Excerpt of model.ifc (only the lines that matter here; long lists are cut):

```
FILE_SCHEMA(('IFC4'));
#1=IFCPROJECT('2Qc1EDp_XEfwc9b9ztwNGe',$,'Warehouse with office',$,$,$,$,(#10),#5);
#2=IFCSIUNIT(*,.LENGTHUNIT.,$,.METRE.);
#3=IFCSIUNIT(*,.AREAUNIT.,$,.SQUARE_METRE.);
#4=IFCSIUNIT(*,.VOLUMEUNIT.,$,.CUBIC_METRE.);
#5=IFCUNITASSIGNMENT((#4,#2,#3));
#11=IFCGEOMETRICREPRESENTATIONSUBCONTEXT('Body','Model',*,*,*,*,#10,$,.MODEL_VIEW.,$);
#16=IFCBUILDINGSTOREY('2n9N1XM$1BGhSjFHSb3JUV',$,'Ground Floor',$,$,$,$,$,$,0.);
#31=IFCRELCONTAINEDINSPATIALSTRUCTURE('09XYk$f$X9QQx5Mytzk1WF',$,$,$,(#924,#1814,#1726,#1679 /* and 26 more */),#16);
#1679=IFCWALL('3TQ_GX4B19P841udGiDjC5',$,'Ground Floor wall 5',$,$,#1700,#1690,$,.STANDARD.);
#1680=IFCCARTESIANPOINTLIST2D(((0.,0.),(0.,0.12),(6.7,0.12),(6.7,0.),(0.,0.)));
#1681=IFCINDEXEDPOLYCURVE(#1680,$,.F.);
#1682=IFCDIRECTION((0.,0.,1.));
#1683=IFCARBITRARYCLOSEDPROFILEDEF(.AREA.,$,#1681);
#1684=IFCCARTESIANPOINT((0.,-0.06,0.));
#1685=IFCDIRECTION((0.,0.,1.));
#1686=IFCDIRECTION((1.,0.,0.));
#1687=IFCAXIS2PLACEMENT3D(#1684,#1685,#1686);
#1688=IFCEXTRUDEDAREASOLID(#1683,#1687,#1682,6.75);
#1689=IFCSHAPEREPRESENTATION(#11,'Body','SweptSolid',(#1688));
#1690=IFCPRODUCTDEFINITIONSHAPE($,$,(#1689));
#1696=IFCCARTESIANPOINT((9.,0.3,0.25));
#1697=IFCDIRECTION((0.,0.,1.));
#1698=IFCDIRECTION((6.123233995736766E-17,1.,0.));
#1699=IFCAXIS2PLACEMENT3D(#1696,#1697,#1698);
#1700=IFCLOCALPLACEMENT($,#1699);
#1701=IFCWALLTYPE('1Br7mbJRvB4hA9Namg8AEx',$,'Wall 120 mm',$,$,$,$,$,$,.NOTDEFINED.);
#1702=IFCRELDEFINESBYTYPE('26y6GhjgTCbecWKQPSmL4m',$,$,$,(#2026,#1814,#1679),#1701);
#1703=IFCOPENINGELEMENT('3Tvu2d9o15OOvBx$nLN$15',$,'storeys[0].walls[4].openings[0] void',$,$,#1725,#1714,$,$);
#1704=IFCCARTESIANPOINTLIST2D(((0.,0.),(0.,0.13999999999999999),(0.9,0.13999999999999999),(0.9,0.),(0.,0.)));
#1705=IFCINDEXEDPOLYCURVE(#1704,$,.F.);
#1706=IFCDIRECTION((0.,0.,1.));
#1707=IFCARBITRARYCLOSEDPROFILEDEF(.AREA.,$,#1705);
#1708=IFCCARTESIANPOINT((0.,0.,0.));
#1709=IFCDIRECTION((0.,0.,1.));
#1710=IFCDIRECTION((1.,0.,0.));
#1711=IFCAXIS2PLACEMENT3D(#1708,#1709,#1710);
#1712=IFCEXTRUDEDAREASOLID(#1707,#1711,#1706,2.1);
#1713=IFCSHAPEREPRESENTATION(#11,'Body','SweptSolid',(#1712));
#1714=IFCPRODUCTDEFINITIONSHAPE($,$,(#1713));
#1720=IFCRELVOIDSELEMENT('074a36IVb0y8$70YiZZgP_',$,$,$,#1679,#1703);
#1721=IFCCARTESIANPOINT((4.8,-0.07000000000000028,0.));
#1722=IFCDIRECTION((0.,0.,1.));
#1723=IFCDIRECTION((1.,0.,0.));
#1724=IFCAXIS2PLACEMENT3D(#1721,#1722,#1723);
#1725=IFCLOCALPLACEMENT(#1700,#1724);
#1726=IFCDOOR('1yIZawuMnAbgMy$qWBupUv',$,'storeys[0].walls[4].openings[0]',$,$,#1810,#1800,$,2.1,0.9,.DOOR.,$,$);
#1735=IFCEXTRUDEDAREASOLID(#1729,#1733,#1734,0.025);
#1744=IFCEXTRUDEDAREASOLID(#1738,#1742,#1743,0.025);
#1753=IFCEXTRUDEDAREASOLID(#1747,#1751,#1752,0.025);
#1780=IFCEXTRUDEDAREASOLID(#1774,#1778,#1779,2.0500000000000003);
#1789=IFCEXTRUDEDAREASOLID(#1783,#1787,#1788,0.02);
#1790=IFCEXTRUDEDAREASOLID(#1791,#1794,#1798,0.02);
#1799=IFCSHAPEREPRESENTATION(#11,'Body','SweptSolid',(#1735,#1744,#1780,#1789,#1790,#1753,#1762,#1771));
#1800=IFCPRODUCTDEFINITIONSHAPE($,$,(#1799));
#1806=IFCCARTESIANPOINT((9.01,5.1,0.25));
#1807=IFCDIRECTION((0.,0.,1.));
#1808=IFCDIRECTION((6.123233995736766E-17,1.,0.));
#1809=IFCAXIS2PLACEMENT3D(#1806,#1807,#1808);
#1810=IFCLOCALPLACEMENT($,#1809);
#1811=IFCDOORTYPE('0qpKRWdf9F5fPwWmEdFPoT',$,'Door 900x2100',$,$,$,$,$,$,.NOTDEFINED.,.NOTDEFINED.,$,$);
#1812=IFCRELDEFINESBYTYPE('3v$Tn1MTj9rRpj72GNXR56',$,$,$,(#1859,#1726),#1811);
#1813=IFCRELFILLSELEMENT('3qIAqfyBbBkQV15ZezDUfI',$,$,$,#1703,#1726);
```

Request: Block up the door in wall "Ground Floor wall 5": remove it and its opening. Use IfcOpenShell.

```python
import ifcopenshell
import ifcopenshell.api.feature
import ifcopenshell.api.root
import ifcopenshell.geom
import ifcopenshell.util.shape

model = ifcopenshell.open("model.ifc")
settings = ifcopenshell.geom.settings()


def volume(element):
    """Net volume in cubic metres, openings subtracted."""
    shape = ifcopenshell.geom.create_shape(settings, element)
    return ifcopenshell.util.shape.get_volume(shape.geometry)


door = model.by_guid("1yIZawuMnAbgMy$qWBupUv")
opening = door.FillsVoids[0].RelatingOpeningElement
wall = opening.VoidsElements[0].RelatingBuildingElement
before = volume(wall)

ifcopenshell.api.root.remove_product(model, product=door)
ifcopenshell.api.feature.remove_feature(model, feature=opening)

after = volume(wall)

print(f"wall volume {before:.3f} -> {after:.3f} m3")

model.write("model_rev.ifc")
```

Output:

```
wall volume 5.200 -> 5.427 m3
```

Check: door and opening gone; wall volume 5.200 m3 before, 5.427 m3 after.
